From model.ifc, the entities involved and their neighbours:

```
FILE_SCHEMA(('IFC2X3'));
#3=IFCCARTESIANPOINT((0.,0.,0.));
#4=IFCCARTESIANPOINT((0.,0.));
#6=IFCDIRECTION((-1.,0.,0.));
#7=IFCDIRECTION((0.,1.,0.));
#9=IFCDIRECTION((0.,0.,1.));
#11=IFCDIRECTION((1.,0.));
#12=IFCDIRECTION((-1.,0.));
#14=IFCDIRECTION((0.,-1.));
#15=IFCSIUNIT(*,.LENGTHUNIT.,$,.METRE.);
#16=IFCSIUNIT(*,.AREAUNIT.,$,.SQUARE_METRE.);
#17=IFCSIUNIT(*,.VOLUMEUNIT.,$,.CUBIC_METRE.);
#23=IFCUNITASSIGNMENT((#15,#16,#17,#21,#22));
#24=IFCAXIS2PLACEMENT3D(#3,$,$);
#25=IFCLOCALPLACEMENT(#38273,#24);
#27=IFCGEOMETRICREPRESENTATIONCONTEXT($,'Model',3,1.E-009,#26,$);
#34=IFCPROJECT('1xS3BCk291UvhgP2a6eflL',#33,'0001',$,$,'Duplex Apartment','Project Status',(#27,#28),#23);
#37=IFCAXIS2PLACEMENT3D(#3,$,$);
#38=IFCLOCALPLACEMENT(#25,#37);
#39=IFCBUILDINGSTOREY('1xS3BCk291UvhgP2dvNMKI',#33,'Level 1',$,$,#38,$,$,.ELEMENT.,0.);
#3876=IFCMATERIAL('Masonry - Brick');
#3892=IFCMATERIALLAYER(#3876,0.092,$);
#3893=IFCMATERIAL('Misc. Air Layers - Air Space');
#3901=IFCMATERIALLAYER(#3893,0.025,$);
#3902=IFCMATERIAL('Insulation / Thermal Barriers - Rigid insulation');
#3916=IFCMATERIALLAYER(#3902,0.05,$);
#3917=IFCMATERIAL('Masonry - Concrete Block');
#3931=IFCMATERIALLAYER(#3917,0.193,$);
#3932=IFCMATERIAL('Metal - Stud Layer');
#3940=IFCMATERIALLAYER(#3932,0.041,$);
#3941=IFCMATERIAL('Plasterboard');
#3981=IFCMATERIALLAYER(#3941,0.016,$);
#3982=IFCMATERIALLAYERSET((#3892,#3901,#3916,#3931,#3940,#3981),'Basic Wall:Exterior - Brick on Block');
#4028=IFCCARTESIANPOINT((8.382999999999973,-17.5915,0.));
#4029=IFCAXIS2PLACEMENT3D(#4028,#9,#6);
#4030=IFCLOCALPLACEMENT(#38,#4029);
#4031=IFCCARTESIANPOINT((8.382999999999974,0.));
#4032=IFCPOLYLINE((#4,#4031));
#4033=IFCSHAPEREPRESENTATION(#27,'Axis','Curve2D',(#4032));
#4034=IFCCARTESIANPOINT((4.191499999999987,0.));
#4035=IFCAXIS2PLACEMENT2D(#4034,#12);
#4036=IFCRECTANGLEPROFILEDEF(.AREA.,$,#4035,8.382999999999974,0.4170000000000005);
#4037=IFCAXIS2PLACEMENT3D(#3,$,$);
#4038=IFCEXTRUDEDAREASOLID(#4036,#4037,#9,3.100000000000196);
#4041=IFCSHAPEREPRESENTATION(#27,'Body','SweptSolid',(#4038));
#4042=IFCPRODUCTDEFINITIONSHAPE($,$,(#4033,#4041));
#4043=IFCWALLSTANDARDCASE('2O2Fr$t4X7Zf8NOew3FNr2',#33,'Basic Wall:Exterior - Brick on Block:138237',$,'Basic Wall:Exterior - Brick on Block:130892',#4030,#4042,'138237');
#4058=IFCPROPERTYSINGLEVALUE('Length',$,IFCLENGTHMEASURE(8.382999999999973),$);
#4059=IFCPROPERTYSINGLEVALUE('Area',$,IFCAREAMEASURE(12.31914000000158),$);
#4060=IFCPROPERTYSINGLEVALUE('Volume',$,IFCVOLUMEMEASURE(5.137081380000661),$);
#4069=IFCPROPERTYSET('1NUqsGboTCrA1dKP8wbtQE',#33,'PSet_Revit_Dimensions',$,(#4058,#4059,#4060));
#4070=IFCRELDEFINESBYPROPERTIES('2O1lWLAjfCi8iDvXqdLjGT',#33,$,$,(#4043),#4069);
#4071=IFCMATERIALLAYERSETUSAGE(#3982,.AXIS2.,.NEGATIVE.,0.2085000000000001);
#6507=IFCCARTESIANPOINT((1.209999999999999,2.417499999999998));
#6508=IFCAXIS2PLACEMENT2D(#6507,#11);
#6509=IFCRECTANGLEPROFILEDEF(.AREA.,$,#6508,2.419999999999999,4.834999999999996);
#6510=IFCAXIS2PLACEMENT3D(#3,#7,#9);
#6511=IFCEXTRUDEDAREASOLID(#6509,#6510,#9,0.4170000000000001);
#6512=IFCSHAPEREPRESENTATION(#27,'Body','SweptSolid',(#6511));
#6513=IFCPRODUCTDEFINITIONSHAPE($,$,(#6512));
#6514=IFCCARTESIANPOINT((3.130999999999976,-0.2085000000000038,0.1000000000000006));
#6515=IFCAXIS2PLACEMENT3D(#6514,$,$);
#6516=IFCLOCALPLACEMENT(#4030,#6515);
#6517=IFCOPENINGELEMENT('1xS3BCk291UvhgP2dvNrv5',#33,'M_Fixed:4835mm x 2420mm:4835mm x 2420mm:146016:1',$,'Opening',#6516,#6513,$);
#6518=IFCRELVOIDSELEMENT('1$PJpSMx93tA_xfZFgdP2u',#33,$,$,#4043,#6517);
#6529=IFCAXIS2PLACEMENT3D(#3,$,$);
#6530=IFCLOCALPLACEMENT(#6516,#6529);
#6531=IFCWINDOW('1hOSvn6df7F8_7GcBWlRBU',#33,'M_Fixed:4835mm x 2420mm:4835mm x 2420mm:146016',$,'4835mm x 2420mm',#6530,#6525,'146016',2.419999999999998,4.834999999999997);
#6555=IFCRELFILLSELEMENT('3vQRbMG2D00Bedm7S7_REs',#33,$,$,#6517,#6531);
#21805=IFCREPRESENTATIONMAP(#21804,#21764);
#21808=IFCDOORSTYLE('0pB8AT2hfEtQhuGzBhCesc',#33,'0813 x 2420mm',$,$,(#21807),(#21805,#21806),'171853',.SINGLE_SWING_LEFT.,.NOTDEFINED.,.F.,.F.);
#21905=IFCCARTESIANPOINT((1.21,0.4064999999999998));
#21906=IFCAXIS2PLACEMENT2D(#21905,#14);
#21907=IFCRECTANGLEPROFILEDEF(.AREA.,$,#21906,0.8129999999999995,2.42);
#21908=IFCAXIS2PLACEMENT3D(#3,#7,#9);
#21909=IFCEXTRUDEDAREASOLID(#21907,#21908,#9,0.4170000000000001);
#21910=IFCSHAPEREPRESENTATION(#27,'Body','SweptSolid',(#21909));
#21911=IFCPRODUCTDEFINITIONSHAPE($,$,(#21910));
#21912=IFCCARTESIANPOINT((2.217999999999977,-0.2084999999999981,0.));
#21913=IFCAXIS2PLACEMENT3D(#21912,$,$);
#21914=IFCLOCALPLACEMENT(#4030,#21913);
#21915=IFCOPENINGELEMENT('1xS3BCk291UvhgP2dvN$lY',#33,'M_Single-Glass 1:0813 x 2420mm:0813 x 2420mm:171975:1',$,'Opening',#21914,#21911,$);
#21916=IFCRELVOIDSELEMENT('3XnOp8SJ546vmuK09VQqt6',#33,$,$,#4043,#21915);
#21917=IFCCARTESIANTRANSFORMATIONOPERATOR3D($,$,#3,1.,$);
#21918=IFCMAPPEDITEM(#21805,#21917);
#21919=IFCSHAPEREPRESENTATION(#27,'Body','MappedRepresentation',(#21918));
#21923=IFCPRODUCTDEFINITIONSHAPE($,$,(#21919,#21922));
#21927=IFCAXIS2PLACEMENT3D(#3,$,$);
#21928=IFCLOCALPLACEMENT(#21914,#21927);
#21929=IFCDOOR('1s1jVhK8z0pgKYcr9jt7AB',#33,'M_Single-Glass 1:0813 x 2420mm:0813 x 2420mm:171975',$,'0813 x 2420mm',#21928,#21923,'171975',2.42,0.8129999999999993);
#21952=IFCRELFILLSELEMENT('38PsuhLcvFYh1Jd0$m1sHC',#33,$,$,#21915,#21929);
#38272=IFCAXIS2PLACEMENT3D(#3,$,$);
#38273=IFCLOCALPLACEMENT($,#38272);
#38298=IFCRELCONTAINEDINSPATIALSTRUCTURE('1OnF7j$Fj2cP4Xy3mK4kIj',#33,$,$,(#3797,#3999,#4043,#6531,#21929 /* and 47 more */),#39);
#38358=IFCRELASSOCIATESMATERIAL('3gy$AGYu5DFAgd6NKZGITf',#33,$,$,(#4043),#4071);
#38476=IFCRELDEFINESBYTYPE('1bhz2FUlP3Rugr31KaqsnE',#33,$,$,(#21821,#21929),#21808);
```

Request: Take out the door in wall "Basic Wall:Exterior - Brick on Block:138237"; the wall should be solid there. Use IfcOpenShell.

```python
import ifcopenshell
import ifcopenshell.api.feature
import ifcopenshell.api.pset
import ifcopenshell.api.root
import ifcopenshell.geom
import ifcopenshell.util.element
import ifcopenshell.util.shape
import ifcopenshell.util.unit

model = ifcopenshell.open("model.ifc")
area_scale = ifcopenshell.util.unit.calculate_unit_scale(model, "AREAUNIT")
volume_scale = ifcopenshell.util.unit.calculate_unit_scale(model, "VOLUMEUNIT")
settings = ifcopenshell.geom.settings()


def volume(element):
    """Net volume in cubic metres, openings subtracted."""
    shape = ifcopenshell.geom.create_shape(settings, element)
    return ifcopenshell.util.shape.get_volume(shape.geometry)


door = model.by_guid("1s1jVhK8z0pgKYcr9jt7AB")
opening = door.FillsVoids[0].RelatingOpeningElement
wall = opening.VoidsElements[0].RelatingBuildingElement
before = volume(wall)

ifcopenshell.api.root.remove_product(model, product=door)
ifcopenshell.api.feature.remove_feature(model, feature=opening)

after = volume(wall)
thickness = 0.417  # wall thickness in metres

# Update the wall's stored quantities.
pset = model.by_id(ifcopenshell.util.element.get_pset(wall, "PSet_Revit_Dimensions", should_inherit=False)["id"])
ifcopenshell.api.pset.edit_pset(model, pset=pset, properties={
    "Area": model.create_entity("IfcAreaMeasure", after / thickness / area_scale),
    "Volume": model.create_entity("IfcVolumeMeasure", after / volume_scale),
})

print(f"wall volume {before:.3f} -> {after:.3f} m3")

model.write("model_v2.ifc")
```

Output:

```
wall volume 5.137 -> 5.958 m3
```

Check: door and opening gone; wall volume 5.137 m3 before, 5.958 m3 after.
